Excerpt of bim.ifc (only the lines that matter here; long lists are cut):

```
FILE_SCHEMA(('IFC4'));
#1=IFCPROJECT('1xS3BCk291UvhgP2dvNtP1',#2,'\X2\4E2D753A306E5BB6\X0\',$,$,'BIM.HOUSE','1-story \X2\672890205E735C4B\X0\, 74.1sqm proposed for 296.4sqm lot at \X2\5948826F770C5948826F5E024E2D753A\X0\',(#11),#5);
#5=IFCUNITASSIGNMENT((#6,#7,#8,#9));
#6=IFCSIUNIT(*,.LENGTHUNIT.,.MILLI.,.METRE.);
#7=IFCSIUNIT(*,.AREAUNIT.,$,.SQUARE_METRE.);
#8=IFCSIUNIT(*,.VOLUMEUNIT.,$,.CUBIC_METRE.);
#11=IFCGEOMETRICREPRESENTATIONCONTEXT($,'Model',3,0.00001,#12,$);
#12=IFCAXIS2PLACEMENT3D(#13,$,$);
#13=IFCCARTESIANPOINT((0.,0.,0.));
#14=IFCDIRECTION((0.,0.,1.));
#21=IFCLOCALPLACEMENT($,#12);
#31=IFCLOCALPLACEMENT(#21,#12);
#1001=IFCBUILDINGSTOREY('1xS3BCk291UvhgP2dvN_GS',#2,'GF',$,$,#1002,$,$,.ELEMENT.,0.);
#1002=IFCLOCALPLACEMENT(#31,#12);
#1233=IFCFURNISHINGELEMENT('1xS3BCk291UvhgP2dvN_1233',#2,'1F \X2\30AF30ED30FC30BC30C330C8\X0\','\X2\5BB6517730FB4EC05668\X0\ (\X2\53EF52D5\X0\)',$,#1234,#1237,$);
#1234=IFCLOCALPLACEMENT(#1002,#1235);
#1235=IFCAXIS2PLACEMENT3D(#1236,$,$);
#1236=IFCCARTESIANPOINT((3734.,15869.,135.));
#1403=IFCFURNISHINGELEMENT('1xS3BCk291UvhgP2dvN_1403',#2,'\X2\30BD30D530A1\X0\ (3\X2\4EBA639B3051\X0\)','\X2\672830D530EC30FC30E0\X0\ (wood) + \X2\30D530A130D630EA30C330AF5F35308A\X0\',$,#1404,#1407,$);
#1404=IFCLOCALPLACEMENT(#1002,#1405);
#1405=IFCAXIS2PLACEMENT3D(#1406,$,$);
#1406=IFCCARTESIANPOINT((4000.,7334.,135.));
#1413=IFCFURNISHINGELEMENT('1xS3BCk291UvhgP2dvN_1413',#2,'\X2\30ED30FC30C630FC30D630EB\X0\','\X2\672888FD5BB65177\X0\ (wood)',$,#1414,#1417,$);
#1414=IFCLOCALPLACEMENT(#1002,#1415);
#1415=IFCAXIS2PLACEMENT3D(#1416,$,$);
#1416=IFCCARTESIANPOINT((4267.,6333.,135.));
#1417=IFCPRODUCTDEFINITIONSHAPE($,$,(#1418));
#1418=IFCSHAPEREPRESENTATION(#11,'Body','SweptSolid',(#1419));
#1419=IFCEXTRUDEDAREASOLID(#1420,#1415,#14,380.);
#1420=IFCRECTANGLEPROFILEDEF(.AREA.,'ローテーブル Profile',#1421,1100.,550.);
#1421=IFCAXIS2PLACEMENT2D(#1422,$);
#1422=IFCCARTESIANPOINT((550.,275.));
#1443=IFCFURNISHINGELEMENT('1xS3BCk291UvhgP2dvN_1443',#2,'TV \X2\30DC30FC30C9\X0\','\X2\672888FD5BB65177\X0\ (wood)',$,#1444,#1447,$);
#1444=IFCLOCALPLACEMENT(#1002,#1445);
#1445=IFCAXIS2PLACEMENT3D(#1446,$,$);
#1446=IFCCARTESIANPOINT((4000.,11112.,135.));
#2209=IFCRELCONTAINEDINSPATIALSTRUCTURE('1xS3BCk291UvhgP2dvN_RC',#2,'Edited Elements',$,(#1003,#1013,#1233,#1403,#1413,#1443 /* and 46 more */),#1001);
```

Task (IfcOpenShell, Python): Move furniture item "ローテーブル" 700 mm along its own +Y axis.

```python
import ifcopenshell
import ifcopenshell.api.geometry
import ifcopenshell.util.placement
import ifcopenshell.util.unit

model = ifcopenshell.open("bim.ifc")
unit_scale = ifcopenshell.util.unit.calculate_unit_scale(model)

item = model.by_guid("1xS3BCk291UvhgP2dvN_1413")
matrix = ifcopenshell.util.placement.get_local_placement(item.ObjectPlacement)
matrix[:3, 3] += matrix[:3, 1] * 0.7 / unit_scale
ifcopenshell.api.geometry.edit_object_placement(model, product=item, matrix=matrix, is_si=False)

print(ifcopenshell.util.placement.get_local_placement(item.ObjectPlacement).round(3) + 0.0)

model.write("bim_edited.ifc")
```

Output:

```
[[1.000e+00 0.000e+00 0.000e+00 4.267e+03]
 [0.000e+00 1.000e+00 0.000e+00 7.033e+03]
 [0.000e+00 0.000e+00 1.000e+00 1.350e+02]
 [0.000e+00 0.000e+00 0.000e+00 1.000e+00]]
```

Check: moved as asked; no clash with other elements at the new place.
